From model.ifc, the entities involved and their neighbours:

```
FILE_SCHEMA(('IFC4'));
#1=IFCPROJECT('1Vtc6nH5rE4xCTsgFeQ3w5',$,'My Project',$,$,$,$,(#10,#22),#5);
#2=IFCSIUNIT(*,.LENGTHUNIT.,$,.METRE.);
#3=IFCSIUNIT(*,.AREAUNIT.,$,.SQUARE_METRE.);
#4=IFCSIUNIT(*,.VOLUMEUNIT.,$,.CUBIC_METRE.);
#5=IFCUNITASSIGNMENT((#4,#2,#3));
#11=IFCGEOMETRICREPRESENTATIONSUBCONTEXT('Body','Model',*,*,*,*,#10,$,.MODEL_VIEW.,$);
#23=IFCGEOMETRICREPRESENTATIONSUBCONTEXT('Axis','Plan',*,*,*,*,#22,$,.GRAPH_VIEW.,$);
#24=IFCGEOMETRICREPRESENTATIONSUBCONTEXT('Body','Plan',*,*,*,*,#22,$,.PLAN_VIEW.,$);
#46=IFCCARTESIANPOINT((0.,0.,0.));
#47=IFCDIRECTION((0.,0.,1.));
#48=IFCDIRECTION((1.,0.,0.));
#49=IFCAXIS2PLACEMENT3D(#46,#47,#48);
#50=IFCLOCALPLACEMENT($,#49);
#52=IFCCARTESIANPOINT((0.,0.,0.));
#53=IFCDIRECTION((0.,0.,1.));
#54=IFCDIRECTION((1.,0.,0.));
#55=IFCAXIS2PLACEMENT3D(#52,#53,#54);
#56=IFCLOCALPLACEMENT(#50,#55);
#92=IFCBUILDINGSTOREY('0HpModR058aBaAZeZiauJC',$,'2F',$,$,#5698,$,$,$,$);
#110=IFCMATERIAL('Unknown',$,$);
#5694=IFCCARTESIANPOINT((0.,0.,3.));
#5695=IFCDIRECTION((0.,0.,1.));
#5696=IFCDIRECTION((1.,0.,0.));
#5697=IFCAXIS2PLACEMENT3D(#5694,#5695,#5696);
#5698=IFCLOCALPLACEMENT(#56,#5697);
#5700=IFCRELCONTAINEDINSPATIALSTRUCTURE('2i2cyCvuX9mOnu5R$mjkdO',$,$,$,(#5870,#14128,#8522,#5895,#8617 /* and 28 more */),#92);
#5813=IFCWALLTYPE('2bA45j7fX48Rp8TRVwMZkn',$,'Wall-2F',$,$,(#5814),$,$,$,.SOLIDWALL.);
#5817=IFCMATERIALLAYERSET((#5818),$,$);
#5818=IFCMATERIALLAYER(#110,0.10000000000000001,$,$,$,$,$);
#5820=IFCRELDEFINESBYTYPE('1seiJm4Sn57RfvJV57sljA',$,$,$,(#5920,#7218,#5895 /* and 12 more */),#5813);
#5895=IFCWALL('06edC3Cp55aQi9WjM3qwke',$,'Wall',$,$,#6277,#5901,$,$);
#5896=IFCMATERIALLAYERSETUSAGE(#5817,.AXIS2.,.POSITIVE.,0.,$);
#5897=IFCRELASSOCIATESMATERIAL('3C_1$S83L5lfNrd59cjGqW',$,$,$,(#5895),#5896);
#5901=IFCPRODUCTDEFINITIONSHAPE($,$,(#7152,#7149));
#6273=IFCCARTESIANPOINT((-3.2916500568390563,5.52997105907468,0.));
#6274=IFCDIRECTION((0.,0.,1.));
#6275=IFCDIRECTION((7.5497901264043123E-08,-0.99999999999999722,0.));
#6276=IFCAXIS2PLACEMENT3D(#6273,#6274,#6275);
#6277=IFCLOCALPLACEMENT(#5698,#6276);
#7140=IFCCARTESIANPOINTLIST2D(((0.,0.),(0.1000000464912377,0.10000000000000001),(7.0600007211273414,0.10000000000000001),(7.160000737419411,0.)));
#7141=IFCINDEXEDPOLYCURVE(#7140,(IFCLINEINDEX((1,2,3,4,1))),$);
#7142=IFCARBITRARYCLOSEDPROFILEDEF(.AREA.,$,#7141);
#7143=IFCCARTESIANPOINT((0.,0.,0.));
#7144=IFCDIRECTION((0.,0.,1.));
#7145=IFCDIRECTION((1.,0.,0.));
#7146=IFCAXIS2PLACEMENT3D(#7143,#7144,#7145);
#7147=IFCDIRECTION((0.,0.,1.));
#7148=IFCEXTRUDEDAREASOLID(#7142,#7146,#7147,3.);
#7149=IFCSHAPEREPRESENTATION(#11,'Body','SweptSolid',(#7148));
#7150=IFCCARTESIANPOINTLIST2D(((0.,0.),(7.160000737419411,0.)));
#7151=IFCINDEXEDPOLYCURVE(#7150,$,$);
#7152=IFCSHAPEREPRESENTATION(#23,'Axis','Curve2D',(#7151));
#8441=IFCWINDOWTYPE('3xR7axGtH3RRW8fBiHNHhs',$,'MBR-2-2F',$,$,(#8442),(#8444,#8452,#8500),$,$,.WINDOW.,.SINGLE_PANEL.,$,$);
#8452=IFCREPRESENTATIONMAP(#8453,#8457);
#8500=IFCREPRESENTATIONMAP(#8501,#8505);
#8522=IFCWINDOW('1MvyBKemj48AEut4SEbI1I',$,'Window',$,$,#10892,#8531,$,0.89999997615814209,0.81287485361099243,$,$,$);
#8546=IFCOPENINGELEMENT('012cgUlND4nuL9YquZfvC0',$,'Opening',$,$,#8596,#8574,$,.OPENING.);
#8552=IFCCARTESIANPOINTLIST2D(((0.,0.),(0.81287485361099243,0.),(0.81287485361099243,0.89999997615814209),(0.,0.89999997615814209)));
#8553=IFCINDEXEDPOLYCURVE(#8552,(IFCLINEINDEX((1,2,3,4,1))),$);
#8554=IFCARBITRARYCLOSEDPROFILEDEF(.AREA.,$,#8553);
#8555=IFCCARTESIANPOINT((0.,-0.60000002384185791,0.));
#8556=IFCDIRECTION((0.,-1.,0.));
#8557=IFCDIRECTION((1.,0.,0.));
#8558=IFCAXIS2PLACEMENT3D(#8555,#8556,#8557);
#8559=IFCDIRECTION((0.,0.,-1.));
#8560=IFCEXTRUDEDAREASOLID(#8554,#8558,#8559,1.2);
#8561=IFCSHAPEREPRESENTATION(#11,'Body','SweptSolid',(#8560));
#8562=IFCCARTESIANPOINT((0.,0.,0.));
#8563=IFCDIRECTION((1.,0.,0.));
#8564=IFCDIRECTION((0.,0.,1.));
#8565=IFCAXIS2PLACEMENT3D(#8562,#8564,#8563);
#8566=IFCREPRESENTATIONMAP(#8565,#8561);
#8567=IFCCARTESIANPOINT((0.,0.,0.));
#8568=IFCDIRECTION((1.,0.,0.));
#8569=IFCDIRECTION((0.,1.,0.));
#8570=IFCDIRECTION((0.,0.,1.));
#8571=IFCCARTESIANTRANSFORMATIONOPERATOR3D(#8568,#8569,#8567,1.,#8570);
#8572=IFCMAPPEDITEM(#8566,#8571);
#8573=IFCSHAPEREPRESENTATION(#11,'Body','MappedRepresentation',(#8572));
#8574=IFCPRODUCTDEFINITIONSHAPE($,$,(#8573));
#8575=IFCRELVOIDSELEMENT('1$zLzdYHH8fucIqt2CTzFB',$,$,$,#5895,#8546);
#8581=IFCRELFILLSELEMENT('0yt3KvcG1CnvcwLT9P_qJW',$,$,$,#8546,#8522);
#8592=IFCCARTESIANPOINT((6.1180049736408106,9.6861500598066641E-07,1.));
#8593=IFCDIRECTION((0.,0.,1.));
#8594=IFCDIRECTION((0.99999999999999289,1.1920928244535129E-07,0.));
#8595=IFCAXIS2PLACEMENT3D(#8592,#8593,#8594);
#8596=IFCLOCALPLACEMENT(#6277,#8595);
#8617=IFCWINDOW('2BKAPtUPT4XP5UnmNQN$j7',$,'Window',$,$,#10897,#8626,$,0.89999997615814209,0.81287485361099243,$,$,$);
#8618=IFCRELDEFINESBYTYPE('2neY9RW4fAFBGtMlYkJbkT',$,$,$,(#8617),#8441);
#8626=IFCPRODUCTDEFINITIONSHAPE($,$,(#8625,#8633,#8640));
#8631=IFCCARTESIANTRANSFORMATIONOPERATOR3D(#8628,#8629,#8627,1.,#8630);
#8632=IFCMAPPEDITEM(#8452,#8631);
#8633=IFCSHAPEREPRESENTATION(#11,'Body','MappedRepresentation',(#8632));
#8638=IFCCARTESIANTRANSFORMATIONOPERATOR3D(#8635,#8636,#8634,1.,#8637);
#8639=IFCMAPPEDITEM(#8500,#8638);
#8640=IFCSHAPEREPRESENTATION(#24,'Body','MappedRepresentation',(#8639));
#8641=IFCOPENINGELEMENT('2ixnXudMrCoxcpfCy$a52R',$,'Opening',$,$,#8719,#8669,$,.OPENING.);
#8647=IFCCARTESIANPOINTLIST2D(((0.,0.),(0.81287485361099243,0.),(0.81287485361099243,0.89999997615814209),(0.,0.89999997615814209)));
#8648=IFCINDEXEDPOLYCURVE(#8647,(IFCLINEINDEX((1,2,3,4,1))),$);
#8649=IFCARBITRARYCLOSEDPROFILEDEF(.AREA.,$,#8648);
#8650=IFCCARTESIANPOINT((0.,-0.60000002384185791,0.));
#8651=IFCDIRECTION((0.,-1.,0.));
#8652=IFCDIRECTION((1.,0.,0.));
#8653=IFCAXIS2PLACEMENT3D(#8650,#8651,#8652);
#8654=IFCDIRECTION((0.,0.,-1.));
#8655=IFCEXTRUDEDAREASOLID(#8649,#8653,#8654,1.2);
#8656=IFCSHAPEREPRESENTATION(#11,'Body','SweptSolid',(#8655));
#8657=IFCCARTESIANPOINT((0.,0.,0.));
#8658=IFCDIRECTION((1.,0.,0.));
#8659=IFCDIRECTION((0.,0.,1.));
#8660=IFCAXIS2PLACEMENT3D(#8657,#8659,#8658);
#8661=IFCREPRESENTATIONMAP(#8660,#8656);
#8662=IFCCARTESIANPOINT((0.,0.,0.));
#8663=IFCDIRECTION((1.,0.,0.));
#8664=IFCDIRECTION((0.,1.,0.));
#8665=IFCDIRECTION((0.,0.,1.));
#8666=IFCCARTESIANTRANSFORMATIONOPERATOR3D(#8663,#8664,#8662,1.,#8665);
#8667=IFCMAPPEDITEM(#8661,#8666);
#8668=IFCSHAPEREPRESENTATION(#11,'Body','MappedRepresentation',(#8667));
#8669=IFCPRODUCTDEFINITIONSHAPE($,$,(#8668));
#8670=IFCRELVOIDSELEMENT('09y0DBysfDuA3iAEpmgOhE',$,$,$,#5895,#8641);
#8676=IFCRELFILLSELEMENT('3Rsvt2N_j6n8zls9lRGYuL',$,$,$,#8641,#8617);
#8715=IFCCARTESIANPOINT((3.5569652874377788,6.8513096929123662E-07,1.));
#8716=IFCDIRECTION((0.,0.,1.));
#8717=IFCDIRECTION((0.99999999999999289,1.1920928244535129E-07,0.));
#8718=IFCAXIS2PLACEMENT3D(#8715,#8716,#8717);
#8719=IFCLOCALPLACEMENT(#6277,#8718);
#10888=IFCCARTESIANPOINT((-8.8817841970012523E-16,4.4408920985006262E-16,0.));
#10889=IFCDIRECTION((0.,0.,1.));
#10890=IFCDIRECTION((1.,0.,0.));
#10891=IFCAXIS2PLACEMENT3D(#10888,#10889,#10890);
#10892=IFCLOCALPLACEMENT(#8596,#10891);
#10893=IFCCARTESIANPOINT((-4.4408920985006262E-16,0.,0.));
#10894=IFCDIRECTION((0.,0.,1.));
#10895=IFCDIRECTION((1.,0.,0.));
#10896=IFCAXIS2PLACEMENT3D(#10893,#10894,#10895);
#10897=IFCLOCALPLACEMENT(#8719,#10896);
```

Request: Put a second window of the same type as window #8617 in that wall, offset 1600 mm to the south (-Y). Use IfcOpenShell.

```python
import ifcopenshell
import ifcopenshell.api.feature
import ifcopenshell.api.geometry
import ifcopenshell.api.root
import ifcopenshell.geom
import ifcopenshell.util.element
import ifcopenshell.util.placement
import ifcopenshell.util.shape
import ifcopenshell.util.unit

model = ifcopenshell.open("model.ifc")
unit_scale = ifcopenshell.util.unit.calculate_unit_scale(model)
settings = ifcopenshell.geom.settings()


def volume(element):
    """Net volume in cubic metres, openings subtracted."""
    shape = ifcopenshell.geom.create_shape(settings, element)
    return ifcopenshell.util.shape.get_volume(shape.geometry)


window = model.by_guid("2BKAPtUPT4XP5UnmNQN$j7")
opening = window.FillsVoids[0].RelatingOpeningElement
wall = opening.VoidsElements[0].RelatingBuildingElement
before = volume(wall)
shift = ifcopenshell.util.placement.get_local_placement(wall.ObjectPlacement)[:3, 0] * 1.6 / unit_scale

# copy_class copies the void relationship, type, container and properties, but no geometry.
new_opening = ifcopenshell.api.root.copy_class(model, product=opening)
new_opening.Representation = ifcopenshell.util.element.copy_deep(
    model, opening.Representation, exclude=["IfcGeometricRepresentationContext", "IfcRepresentationMap"]
)
new_window = ifcopenshell.api.root.copy_class(model, product=window)
new_window.Representation = ifcopenshell.util.element.copy_deep(
    model, window.Representation, exclude=["IfcGeometricRepresentationContext", "IfcRepresentationMap"]
)
ifcopenshell.api.feature.add_filling(model, opening=new_opening, element=new_window)

for old, new in ((opening, new_opening), (window, new_window)):
    matrix = ifcopenshell.util.placement.get_local_placement(old.ObjectPlacement)
    matrix[:3, 3] += shift
    ifcopenshell.api.geometry.edit_object_placement(model, product=new, matrix=matrix, is_si=False)

after = volume(wall)

print(f"wall volume {before:.3f} -> {after:.3f} m3")

model.write("model_updated.ifc")
```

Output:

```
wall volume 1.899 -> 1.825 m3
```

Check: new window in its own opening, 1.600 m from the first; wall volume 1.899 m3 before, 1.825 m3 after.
